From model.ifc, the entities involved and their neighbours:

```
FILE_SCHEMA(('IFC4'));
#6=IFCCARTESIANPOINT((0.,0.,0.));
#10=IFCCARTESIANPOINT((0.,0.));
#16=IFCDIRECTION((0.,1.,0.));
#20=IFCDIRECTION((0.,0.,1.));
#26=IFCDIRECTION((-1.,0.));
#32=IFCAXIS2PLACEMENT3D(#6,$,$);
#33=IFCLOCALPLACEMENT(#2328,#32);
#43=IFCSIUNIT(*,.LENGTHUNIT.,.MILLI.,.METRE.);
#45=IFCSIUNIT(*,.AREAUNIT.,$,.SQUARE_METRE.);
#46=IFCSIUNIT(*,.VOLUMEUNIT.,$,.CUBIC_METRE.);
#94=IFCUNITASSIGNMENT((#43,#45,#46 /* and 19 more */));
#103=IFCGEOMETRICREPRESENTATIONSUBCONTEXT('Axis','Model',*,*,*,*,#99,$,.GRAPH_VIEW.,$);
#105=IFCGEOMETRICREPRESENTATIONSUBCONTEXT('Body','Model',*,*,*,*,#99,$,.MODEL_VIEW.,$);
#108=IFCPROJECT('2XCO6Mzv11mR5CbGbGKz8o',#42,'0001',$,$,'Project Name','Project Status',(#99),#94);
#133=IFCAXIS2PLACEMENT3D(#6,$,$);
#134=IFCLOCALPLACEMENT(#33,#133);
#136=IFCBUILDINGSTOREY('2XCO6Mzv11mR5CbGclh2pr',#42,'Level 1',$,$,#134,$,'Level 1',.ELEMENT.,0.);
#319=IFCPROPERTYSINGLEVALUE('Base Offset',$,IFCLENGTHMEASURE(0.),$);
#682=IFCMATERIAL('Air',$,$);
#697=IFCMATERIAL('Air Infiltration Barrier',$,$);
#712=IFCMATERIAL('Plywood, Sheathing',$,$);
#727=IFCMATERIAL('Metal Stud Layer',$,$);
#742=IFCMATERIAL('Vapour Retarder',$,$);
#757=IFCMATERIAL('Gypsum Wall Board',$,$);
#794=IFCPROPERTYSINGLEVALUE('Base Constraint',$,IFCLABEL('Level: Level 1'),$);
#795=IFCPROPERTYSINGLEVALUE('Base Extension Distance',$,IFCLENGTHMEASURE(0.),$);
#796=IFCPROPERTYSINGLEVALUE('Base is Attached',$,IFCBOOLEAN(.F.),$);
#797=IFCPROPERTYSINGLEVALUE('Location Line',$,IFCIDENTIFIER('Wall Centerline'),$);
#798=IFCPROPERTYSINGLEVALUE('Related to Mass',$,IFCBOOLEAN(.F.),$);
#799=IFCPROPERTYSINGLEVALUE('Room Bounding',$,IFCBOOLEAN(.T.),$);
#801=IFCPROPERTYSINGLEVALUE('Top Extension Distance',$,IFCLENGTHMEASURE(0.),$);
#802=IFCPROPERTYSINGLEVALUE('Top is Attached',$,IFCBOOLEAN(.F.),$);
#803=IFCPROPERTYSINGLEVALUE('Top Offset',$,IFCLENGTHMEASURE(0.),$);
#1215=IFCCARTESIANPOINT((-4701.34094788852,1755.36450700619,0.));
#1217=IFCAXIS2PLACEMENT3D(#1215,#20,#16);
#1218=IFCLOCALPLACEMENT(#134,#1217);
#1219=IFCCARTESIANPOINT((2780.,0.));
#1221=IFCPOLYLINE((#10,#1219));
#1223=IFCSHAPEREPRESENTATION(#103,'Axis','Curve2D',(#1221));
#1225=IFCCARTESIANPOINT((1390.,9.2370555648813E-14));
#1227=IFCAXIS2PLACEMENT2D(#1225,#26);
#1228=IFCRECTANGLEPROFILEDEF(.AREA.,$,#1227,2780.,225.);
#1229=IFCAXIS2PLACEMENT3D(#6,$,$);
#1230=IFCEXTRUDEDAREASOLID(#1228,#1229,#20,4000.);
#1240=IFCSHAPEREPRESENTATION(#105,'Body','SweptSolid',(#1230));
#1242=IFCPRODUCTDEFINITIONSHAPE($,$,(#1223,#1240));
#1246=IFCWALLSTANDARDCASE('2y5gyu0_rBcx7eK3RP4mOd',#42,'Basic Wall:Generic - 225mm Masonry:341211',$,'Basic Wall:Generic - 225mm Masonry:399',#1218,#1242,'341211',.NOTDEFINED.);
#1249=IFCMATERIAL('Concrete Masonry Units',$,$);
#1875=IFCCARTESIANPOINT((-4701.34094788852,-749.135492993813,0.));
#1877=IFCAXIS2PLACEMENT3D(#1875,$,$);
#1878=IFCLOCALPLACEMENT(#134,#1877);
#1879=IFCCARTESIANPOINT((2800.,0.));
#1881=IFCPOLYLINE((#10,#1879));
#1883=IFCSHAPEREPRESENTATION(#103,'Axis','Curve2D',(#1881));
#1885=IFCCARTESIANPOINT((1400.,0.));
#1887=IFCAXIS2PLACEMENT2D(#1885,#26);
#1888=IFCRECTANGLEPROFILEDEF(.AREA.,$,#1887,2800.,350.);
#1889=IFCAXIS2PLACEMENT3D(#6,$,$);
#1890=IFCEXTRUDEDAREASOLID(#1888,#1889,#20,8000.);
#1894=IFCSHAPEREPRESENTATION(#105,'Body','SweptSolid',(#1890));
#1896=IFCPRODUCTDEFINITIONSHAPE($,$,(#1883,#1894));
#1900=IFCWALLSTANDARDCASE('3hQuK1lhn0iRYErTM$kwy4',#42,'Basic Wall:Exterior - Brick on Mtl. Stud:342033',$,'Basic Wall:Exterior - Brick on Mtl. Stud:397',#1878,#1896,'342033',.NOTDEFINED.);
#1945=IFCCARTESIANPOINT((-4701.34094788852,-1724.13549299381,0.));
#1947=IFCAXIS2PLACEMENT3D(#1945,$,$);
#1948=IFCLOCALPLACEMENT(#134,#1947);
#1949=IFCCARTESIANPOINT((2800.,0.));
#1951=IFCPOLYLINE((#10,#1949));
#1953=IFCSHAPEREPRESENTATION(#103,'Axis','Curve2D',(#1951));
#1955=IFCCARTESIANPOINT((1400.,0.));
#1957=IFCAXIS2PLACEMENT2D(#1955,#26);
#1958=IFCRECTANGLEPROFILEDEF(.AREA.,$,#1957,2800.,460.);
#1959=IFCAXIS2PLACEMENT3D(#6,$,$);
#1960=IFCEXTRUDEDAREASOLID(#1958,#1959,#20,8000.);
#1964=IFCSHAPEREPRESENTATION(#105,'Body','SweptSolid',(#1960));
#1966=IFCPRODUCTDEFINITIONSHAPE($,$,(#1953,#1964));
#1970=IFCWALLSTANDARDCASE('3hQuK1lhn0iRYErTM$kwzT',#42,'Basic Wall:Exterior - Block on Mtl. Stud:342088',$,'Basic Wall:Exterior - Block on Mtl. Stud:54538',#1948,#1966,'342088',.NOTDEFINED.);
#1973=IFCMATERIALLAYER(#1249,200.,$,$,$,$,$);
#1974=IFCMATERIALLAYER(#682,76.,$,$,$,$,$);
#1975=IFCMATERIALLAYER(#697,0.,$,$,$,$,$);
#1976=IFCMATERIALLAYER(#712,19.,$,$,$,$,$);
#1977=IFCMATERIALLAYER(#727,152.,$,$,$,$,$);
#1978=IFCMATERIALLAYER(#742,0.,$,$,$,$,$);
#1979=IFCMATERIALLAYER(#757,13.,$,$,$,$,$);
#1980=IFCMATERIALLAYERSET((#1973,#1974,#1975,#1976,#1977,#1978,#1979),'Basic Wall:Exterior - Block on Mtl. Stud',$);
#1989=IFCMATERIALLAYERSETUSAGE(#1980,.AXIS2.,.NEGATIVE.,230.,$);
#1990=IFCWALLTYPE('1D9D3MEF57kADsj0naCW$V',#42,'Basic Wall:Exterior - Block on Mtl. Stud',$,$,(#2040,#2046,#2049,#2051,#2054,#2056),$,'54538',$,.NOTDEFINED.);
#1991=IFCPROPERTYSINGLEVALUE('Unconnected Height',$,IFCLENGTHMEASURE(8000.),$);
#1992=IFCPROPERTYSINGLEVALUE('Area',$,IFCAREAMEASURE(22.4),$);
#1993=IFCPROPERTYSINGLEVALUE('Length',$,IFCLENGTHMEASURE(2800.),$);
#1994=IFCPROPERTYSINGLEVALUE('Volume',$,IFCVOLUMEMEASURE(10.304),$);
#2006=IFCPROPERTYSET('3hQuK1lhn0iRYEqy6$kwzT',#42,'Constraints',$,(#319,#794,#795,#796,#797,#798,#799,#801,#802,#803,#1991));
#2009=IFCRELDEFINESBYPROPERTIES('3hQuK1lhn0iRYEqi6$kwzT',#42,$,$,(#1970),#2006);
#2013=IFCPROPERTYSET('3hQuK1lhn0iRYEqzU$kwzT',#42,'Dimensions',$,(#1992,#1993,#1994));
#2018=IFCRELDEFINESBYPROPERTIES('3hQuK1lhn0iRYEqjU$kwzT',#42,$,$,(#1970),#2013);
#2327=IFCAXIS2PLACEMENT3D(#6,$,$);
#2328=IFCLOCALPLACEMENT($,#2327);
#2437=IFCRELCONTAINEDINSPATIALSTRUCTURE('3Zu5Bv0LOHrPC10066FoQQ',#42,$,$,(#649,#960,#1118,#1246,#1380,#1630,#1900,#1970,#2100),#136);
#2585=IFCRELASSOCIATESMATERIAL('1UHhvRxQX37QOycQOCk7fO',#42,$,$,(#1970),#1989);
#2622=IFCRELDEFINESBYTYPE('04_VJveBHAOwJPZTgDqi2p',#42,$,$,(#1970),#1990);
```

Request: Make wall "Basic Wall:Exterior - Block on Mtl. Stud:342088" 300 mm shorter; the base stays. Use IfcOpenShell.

```python
import ifcopenshell
import ifcopenshell.api.pset
import ifcopenshell.geom
import ifcopenshell.util.element
import ifcopenshell.util.representation
import ifcopenshell.util.shape
import ifcopenshell.util.unit

model = ifcopenshell.open("model.ifc")
area_scale = ifcopenshell.util.unit.calculate_unit_scale(model, "AREAUNIT")
volume_scale = ifcopenshell.util.unit.calculate_unit_scale(model, "VOLUMEUNIT")
settings = ifcopenshell.geom.settings()


def volume(element):
    """Net volume in cubic metres, openings subtracted."""
    shape = ifcopenshell.geom.create_shape(settings, element)
    return ifcopenshell.util.shape.get_volume(shape.geometry)


wall = model.by_id(1970)
before = volume(wall)

body = ifcopenshell.util.representation.get_representation(wall, "Model", "Body")
solid = body.Items[0]
old_height = solid.Depth
solid.Depth -= 300.0
after = volume(wall)
thickness = 0.46  # wall thickness in metres

# Update the stored height, areas and volumes.
pset = model.by_id(ifcopenshell.util.element.get_pset(wall, "Constraints", should_inherit=False)["id"])
ifcopenshell.api.pset.edit_pset(model, pset=pset, properties={
    "Unconnected Height": model.create_entity("IfcLengthMeasure", solid.Depth),
})
pset = model.by_id(ifcopenshell.util.element.get_pset(wall, "Dimensions", should_inherit=False)["id"])
ifcopenshell.api.pset.edit_pset(model, pset=pset, properties={
    "Area": model.create_entity("IfcAreaMeasure", after / thickness / area_scale),
    "Volume": model.create_entity("IfcVolumeMeasure", after / volume_scale),
})

print(f"height {old_height:g} -> {solid.Depth:g}, volume {before:.3f} -> {after:.3f} m3")

model.write("model_edited.ifc")
```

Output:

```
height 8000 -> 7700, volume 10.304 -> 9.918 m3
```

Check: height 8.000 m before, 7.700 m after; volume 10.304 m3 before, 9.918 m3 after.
